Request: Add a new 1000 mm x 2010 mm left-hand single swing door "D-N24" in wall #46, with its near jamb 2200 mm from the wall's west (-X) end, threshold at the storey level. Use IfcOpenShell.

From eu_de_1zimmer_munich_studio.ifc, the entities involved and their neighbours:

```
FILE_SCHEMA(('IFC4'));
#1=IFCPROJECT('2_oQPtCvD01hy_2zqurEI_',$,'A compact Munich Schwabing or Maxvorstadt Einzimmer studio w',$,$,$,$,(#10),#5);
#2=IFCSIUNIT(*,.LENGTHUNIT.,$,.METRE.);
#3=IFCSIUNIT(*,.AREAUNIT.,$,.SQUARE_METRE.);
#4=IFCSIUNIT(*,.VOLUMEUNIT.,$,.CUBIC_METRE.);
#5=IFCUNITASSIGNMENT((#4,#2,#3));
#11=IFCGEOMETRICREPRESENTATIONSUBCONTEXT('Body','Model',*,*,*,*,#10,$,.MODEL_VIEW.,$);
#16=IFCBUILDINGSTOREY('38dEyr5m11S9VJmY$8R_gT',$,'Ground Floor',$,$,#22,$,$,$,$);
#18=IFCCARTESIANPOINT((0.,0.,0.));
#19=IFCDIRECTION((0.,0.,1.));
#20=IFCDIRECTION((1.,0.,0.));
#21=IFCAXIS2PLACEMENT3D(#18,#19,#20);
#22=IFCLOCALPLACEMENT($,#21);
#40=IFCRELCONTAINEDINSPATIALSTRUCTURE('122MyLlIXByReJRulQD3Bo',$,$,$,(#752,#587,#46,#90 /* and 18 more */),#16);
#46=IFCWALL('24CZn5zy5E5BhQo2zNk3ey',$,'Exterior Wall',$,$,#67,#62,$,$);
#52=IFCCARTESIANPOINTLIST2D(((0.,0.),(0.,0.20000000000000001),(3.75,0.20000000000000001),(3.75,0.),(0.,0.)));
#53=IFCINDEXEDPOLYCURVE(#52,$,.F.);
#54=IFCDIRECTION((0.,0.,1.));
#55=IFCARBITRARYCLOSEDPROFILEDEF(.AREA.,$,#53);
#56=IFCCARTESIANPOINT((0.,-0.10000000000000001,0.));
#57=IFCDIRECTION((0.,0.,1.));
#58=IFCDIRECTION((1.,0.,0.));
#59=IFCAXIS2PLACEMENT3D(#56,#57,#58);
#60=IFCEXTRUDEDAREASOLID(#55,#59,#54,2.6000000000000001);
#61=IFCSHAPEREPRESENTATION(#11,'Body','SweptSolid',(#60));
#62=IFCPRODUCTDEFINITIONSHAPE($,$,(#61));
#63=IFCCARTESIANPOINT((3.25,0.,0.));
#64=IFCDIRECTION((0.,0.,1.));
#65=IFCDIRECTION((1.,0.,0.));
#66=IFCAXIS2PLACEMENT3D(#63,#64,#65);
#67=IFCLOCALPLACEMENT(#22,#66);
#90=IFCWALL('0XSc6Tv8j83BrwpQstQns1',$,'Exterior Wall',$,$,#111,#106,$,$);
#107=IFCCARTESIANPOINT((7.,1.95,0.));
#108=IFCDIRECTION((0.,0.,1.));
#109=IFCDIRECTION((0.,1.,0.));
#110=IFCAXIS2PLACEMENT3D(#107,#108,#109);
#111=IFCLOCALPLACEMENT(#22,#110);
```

```python
import numpy as np
import ifcopenshell
import ifcopenshell.api.feature
import ifcopenshell.api.geometry
import ifcopenshell.api.root
import ifcopenshell.api.spatial
import ifcopenshell.geom
import ifcopenshell.util.element
import ifcopenshell.util.placement
import ifcopenshell.util.representation
import ifcopenshell.util.shape
import ifcopenshell.util.unit

model = ifcopenshell.open("eu_de_1zimmer_munich_studio.ifc")
unit_scale = ifcopenshell.util.unit.calculate_unit_scale(model)
settings = ifcopenshell.geom.settings()


def volume(element):
    """Net volume in cubic metres, openings subtracted."""
    shape = ifcopenshell.geom.create_shape(settings, element)
    return ifcopenshell.util.shape.get_volume(shape.geometry)


wall = model.by_guid("24CZn5zy5E5BhQo2zNk3ey")
storey = ifcopenshell.util.element.get_container(wall, ifc_class="IfcBuildingStorey")
context = ifcopenshell.util.representation.get_context(model, "Model", "Body", "MODEL_VIEW")
before = volume(wall)

width, height, from_end, sill = 1, 2.01, 2.2, 0.0  # metres

# The wall runs along its own X axis, and the end named is its -X end.
wall_shape = ifcopenshell.geom.create_shape(settings, wall)
x, y, z = ifcopenshell.util.shape.get_vertices(wall_shape.geometry).T
start = x.min() + from_end
face, thickness = float(y.min()), float(y.max() - y.min())
wall_matrix = ifcopenshell.util.placement.get_local_placement(wall.ObjectPlacement)
level = ifcopenshell.util.placement.get_local_placement(storey.ObjectPlacement)[2, 3]


def in_wall(x, y):
    """Placement at x, y metres in the wall's axes, at sill height."""
    matrix = wall_matrix.copy()
    matrix[:, 3] = wall_matrix @ np.array([x / unit_scale, y / unit_scale, 0.0, 1.0])
    matrix[2, 3] = level + sill / unit_scale
    return matrix


# Opening: a box that overshoots both wall faces by 50 mm.
opening = ifcopenshell.api.root.create_entity(model, ifc_class="IfcOpeningElement", predefined_type="OPENING")
box = ifcopenshell.api.geometry.add_wall_representation(
    model, context=context, length=width, height=height, thickness=thickness + 0.1
)
ifcopenshell.api.geometry.assign_representation(model, product=opening, representation=box)
ifcopenshell.api.geometry.edit_object_placement(model, product=opening, matrix=in_wall(start, face - 0.05), is_si=False)
ifcopenshell.api.feature.add_feature(model, feature=opening, element=wall)

door = ifcopenshell.api.root.create_entity(model, ifc_class="IfcDoor", name="D-N24", predefined_type="DOOR")
door.OverallWidth, door.OverallHeight = width / unit_scale, height / unit_scale
door.OperationType = "SINGLE_SWING_LEFT"
body = ifcopenshell.api.geometry.add_door_representation(
    model,
    context=context,
    overall_width=door.OverallWidth,
    overall_height=door.OverallHeight,
    operation_type="SINGLE_SWING_LEFT",
    lining_properties={"LiningDepth": thickness / unit_scale, "ThresholdDepth": thickness / unit_scale},
)
ifcopenshell.api.geometry.assign_representation(model, product=door, representation=body)
ifcopenshell.api.spatial.assign_container(model, products=[door], relating_structure=storey)
ifcopenshell.api.feature.add_filling(model, opening=opening, element=door)

# The lining spans the wall, so the door starts at the wall face.
ifcopenshell.api.geometry.edit_object_placement(model, product=door, matrix=in_wall(start, face), is_si=False)

after = volume(wall)

print(f"wall volume {before:.3f} -> {after:.3f} m3")

model.write("eu_de_1zimmer_munich_studio-out.ifc")
```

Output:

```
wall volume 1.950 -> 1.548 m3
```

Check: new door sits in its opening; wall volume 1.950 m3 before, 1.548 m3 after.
